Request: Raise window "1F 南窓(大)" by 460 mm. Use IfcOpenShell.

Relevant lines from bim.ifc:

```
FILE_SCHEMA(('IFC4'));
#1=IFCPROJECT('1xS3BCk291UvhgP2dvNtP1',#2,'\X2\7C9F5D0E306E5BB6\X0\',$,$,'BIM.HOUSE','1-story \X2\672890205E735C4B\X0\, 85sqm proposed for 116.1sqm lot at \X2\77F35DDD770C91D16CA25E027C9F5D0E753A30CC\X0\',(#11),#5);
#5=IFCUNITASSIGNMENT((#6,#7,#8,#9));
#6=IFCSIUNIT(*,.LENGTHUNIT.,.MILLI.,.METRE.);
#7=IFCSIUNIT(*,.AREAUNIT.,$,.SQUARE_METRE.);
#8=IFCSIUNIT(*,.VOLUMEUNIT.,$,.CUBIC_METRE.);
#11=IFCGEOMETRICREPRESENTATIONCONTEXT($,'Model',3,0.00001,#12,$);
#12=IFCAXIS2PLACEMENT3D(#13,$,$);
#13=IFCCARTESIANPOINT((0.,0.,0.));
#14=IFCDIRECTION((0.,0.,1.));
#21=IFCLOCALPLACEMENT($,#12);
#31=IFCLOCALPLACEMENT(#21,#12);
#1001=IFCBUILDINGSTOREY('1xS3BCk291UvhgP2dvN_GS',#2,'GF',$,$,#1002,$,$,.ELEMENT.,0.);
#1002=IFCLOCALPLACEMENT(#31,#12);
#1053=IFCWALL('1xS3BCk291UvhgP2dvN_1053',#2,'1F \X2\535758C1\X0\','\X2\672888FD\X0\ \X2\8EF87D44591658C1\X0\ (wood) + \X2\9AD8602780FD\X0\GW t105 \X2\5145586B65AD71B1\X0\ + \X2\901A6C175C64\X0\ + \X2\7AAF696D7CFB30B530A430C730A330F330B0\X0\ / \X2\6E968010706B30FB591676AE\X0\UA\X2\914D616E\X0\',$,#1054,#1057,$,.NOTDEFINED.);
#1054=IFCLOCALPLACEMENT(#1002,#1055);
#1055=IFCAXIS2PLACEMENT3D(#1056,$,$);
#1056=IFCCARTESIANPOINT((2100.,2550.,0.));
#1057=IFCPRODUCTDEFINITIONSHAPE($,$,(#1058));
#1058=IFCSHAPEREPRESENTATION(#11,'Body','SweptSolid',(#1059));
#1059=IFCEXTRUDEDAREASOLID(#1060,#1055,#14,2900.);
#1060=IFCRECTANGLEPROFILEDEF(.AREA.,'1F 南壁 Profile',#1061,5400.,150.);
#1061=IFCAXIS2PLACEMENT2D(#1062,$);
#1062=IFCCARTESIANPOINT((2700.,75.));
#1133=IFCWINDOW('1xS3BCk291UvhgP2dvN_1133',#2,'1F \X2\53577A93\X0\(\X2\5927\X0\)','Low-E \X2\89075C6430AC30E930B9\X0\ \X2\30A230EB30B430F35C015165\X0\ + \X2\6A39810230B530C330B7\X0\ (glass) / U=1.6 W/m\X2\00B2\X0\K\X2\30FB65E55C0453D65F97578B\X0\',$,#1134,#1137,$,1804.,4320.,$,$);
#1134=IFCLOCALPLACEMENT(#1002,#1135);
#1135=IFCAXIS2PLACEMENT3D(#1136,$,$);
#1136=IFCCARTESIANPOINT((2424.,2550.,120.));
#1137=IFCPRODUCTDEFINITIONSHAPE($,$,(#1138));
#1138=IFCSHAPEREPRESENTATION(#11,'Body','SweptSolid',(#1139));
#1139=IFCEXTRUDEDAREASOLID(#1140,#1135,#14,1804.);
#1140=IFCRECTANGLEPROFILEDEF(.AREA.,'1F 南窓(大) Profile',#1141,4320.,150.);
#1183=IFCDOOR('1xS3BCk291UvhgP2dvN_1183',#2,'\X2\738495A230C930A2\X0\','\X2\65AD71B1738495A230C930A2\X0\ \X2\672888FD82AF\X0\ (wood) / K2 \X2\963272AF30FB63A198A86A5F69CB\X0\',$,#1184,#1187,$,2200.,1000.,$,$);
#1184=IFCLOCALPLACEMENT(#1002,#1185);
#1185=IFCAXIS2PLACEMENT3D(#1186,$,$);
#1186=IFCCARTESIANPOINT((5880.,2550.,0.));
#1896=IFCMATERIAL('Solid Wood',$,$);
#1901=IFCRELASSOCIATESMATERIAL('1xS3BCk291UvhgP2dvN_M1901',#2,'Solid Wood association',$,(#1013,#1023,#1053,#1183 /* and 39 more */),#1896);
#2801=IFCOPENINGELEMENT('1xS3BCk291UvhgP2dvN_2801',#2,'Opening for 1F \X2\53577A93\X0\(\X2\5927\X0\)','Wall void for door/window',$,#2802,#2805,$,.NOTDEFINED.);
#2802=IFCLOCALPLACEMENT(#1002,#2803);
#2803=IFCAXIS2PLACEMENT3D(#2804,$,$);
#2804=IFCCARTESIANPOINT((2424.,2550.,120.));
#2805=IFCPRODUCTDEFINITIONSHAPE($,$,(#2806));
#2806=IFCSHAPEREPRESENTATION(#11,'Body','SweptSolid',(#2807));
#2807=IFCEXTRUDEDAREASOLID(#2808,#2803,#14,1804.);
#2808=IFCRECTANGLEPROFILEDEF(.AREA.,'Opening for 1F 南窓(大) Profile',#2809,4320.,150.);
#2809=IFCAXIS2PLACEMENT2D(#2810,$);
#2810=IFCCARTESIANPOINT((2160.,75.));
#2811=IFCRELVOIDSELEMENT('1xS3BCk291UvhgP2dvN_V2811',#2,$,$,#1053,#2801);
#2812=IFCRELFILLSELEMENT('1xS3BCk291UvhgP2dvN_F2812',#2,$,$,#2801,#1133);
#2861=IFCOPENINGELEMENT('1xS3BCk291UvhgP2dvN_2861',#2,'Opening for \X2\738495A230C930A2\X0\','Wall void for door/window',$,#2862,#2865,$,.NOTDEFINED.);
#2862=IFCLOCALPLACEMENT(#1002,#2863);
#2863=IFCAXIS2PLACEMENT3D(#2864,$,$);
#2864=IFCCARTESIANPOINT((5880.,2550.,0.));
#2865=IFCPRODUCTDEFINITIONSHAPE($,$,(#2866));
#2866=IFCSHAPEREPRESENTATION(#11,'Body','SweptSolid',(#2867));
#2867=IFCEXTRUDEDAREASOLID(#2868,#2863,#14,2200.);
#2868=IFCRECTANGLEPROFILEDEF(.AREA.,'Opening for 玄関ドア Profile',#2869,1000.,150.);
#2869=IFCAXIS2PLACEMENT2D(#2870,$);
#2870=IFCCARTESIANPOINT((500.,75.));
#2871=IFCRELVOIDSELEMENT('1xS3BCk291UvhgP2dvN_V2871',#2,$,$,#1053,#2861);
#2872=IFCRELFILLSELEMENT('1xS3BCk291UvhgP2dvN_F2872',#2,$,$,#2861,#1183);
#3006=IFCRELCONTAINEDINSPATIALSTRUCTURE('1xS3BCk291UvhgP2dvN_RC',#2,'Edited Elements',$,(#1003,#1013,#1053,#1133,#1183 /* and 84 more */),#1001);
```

```python
import numpy as np
import ifcopenshell
import ifcopenshell.api.geometry
import ifcopenshell.util.placement
import ifcopenshell.util.unit

model = ifcopenshell.open("bim.ifc")
unit_scale = ifcopenshell.util.unit.calculate_unit_scale(model)

window = model.by_guid("1xS3BCk291UvhgP2dvN_1133")
opening = window.FillsVoids[0].RelatingOpeningElement
dz = 0.46 / unit_scale

shift = np.array([0.0, 0.0, dz])
# The window is not placed relative to its opening, so move both.
for product in (opening, window):
    matrix = ifcopenshell.util.placement.get_local_placement(product.ObjectPlacement)
    matrix[:3, 3] += shift
    ifcopenshell.api.geometry.edit_object_placement(model, product=product, matrix=matrix, is_si=False)

print(f"moved by {dz * unit_scale:+.3f} m")

model.write("bim_edited.ifc")
```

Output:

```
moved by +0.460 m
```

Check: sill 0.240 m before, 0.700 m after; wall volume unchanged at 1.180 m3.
